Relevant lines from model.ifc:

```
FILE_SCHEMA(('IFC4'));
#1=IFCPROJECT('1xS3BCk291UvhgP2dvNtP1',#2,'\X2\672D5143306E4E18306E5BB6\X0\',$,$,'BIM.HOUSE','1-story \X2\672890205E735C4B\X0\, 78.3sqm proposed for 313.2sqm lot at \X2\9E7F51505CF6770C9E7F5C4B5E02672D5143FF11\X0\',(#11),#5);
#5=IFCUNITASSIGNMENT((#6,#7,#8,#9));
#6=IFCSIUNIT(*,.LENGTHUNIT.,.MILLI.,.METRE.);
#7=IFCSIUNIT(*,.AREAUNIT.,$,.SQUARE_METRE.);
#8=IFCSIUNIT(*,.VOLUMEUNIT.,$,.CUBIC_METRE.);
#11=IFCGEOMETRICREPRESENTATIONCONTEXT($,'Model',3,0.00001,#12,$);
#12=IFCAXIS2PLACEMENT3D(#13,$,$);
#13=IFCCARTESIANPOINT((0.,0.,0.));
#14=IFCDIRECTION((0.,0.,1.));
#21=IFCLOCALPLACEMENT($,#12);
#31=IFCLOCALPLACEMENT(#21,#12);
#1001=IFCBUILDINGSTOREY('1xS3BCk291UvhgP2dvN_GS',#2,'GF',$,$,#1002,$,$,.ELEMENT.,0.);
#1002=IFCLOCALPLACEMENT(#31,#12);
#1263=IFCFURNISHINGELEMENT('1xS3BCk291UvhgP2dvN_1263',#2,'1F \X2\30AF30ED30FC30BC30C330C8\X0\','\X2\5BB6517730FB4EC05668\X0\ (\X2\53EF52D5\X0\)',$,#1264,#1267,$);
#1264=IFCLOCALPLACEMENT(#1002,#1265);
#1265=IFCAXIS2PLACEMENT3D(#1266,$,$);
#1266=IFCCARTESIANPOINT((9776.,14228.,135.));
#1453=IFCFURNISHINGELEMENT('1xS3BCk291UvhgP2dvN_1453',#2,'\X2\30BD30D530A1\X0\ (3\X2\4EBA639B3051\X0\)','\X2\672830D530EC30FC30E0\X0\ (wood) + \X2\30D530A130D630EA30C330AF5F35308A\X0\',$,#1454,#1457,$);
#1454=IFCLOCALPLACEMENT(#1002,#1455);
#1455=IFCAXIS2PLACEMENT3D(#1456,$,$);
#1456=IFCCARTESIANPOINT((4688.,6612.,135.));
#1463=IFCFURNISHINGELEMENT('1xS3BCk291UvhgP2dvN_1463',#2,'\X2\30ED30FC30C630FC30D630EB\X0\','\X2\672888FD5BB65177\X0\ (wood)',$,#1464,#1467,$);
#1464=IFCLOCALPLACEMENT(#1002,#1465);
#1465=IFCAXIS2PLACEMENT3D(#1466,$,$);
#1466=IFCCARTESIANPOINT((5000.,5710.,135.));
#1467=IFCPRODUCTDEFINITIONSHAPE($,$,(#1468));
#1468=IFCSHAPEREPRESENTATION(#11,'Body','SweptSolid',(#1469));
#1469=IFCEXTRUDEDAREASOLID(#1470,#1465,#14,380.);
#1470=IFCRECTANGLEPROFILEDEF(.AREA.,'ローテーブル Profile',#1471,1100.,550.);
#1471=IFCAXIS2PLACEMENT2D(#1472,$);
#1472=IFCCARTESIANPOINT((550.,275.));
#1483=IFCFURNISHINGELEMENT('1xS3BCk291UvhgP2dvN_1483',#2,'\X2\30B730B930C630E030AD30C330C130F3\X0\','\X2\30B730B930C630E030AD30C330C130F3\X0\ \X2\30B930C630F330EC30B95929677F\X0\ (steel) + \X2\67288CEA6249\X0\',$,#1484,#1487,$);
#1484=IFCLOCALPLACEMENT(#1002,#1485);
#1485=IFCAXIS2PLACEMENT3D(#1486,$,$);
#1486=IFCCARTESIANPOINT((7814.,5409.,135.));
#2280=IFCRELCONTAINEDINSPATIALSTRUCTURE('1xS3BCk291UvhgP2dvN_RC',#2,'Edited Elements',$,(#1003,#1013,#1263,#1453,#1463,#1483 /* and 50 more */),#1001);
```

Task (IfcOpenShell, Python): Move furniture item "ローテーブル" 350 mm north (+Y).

```python
import ifcopenshell
import ifcopenshell.api.geometry
import ifcopenshell.util.placement

model = ifcopenshell.open("model.ifc")

item = model.by_guid("1xS3BCk291UvhgP2dvN_1463")
matrix = ifcopenshell.util.placement.get_local_placement(item.ObjectPlacement)
matrix[1, 3] += 350.0
ifcopenshell.api.geometry.edit_object_placement(model, product=item, matrix=matrix, is_si=False)

print(ifcopenshell.util.placement.get_local_placement(item.ObjectPlacement).round(3) + 0.0)

model.write("model_rev.ifc")
```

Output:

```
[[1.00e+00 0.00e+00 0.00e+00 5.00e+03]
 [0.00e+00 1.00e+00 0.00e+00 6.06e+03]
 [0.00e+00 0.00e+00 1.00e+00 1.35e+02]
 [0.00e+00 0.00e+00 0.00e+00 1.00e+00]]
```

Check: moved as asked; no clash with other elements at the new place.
